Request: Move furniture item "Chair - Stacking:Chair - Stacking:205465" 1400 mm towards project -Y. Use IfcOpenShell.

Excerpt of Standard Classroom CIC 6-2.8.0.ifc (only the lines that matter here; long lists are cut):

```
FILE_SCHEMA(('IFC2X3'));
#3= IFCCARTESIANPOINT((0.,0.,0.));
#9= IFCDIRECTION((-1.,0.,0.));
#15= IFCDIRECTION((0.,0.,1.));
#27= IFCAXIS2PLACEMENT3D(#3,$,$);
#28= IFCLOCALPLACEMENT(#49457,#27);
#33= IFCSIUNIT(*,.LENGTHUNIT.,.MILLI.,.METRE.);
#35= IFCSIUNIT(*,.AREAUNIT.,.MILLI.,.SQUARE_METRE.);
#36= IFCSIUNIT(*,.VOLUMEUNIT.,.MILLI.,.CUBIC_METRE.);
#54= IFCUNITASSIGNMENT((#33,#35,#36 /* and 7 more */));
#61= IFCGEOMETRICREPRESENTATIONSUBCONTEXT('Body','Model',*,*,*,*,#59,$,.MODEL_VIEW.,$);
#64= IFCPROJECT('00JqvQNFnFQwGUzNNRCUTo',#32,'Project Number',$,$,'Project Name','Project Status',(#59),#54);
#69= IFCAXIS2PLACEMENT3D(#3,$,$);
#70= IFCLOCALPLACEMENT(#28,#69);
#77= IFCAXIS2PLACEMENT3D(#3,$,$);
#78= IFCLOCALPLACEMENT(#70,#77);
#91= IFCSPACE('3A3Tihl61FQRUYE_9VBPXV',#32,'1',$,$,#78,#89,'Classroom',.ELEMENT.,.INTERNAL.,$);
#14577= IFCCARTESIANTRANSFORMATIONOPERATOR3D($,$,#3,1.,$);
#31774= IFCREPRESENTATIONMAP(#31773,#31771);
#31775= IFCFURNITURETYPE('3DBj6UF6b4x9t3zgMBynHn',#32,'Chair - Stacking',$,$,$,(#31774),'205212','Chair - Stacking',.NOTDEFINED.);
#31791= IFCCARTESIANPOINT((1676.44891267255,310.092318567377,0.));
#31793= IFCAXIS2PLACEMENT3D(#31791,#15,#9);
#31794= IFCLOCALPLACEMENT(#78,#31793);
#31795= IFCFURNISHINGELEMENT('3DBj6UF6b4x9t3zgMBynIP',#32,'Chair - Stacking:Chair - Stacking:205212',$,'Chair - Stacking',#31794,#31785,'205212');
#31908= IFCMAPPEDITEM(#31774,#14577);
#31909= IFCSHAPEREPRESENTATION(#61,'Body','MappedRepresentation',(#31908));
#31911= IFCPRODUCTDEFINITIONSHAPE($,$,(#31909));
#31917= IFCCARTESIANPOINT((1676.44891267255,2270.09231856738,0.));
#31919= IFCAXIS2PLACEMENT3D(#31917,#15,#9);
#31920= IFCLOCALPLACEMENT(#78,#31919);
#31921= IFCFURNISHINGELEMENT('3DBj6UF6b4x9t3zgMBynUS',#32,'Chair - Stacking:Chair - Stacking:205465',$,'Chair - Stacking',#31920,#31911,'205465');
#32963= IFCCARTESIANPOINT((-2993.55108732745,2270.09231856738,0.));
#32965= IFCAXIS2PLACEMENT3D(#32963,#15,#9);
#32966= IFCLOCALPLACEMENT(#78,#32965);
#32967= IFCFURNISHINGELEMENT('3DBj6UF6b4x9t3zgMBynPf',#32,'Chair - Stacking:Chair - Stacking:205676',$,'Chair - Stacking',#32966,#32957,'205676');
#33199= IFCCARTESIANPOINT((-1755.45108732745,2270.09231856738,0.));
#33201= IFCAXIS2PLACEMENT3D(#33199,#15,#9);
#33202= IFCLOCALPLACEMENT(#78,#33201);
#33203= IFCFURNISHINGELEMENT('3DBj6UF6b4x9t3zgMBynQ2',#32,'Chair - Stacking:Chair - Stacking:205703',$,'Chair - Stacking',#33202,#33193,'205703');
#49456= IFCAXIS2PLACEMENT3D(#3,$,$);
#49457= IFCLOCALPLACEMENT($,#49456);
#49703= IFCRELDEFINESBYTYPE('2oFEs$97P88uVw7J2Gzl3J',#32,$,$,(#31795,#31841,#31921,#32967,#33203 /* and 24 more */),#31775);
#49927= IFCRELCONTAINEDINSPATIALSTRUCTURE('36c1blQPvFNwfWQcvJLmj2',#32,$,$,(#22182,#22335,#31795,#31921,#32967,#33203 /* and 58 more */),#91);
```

```python
import ifcopenshell
import ifcopenshell.api.geometry
import ifcopenshell.util.placement
import ifcopenshell.util.unit

model = ifcopenshell.open("Standard Classroom CIC 6-2.8.0.ifc")
unit_scale = ifcopenshell.util.unit.calculate_unit_scale(model)

item = model.by_guid("3DBj6UF6b4x9t3zgMBynUS")
matrix = ifcopenshell.util.placement.get_local_placement(item.ObjectPlacement)
matrix[1, 3] -= 1.4 / unit_scale
ifcopenshell.api.geometry.edit_object_placement(model, product=item, matrix=matrix, is_si=False)

print(ifcopenshell.util.placement.get_local_placement(item.ObjectPlacement).round(3) + 0.0)

model.write("Standard Classroom CIC 6-2.8.0_updated.ifc")
```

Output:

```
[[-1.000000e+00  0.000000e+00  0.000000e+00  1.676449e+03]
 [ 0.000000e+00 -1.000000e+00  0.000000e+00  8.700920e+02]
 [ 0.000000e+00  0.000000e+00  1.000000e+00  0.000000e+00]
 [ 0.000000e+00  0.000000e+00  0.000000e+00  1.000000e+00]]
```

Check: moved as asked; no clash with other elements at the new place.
